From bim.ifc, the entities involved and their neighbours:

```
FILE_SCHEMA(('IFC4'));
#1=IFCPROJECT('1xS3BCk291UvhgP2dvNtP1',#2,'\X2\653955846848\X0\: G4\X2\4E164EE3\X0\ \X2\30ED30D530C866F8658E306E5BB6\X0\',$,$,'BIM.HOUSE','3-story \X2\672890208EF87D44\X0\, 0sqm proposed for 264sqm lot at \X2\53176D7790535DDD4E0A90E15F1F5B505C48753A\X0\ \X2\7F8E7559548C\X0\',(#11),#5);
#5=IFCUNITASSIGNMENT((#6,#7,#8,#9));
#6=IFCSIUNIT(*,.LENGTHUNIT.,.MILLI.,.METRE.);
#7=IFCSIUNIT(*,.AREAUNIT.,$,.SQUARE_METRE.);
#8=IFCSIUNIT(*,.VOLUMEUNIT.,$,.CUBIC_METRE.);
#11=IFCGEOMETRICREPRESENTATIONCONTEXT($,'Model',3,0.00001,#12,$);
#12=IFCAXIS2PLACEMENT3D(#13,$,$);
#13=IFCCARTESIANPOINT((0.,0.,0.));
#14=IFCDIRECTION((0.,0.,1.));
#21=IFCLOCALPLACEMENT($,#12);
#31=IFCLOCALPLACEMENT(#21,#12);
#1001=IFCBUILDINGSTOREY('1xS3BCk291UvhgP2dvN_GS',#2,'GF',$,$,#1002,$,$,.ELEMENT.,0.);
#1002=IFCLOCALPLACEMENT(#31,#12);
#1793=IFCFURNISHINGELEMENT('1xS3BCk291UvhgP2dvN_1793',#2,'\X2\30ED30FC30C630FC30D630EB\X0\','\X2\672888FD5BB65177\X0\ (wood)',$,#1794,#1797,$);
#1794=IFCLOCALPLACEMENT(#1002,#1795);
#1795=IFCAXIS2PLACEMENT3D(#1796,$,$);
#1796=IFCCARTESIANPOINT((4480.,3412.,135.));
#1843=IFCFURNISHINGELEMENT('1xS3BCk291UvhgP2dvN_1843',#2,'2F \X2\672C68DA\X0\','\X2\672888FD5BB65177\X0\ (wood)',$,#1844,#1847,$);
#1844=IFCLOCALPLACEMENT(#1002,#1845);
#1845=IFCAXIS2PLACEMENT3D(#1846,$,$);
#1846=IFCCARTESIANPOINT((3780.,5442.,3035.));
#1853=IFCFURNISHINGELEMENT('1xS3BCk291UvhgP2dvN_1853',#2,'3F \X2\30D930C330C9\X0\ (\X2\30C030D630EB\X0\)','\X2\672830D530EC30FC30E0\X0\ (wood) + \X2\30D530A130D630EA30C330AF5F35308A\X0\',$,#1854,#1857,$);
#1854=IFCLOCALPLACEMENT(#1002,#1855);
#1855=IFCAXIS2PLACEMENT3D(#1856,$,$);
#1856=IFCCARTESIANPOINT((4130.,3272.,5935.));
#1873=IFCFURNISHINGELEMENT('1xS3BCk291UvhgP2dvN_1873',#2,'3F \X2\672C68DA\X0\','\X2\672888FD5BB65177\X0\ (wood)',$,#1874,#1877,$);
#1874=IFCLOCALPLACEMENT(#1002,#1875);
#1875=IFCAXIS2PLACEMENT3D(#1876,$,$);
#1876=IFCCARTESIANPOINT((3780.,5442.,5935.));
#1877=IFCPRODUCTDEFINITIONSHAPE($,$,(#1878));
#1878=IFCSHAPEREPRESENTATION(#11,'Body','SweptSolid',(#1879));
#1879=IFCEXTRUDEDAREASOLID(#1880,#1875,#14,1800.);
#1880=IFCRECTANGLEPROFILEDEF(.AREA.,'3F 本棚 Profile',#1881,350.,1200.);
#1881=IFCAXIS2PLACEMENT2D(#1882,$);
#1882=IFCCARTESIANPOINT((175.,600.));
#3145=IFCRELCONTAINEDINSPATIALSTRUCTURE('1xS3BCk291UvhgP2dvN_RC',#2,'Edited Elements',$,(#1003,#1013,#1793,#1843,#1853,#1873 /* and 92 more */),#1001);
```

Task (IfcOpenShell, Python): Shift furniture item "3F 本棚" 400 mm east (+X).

```python
import ifcopenshell
import ifcopenshell.api.geometry
import ifcopenshell.util.placement

model = ifcopenshell.open("bim.ifc")

item = model.by_guid("1xS3BCk291UvhgP2dvN_1873")
matrix = ifcopenshell.util.placement.get_local_placement(item.ObjectPlacement)
matrix[0, 3] += 400.0
ifcopenshell.api.geometry.edit_object_placement(model, product=item, matrix=matrix, is_si=False)

print(ifcopenshell.util.placement.get_local_placement(item.ObjectPlacement).round(3) + 0.0)

model.write("bim_v2.ifc")
```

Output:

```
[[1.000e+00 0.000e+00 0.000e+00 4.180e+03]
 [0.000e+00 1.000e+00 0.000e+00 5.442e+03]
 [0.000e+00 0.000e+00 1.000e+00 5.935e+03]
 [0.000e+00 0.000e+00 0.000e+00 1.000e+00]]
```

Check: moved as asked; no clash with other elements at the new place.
